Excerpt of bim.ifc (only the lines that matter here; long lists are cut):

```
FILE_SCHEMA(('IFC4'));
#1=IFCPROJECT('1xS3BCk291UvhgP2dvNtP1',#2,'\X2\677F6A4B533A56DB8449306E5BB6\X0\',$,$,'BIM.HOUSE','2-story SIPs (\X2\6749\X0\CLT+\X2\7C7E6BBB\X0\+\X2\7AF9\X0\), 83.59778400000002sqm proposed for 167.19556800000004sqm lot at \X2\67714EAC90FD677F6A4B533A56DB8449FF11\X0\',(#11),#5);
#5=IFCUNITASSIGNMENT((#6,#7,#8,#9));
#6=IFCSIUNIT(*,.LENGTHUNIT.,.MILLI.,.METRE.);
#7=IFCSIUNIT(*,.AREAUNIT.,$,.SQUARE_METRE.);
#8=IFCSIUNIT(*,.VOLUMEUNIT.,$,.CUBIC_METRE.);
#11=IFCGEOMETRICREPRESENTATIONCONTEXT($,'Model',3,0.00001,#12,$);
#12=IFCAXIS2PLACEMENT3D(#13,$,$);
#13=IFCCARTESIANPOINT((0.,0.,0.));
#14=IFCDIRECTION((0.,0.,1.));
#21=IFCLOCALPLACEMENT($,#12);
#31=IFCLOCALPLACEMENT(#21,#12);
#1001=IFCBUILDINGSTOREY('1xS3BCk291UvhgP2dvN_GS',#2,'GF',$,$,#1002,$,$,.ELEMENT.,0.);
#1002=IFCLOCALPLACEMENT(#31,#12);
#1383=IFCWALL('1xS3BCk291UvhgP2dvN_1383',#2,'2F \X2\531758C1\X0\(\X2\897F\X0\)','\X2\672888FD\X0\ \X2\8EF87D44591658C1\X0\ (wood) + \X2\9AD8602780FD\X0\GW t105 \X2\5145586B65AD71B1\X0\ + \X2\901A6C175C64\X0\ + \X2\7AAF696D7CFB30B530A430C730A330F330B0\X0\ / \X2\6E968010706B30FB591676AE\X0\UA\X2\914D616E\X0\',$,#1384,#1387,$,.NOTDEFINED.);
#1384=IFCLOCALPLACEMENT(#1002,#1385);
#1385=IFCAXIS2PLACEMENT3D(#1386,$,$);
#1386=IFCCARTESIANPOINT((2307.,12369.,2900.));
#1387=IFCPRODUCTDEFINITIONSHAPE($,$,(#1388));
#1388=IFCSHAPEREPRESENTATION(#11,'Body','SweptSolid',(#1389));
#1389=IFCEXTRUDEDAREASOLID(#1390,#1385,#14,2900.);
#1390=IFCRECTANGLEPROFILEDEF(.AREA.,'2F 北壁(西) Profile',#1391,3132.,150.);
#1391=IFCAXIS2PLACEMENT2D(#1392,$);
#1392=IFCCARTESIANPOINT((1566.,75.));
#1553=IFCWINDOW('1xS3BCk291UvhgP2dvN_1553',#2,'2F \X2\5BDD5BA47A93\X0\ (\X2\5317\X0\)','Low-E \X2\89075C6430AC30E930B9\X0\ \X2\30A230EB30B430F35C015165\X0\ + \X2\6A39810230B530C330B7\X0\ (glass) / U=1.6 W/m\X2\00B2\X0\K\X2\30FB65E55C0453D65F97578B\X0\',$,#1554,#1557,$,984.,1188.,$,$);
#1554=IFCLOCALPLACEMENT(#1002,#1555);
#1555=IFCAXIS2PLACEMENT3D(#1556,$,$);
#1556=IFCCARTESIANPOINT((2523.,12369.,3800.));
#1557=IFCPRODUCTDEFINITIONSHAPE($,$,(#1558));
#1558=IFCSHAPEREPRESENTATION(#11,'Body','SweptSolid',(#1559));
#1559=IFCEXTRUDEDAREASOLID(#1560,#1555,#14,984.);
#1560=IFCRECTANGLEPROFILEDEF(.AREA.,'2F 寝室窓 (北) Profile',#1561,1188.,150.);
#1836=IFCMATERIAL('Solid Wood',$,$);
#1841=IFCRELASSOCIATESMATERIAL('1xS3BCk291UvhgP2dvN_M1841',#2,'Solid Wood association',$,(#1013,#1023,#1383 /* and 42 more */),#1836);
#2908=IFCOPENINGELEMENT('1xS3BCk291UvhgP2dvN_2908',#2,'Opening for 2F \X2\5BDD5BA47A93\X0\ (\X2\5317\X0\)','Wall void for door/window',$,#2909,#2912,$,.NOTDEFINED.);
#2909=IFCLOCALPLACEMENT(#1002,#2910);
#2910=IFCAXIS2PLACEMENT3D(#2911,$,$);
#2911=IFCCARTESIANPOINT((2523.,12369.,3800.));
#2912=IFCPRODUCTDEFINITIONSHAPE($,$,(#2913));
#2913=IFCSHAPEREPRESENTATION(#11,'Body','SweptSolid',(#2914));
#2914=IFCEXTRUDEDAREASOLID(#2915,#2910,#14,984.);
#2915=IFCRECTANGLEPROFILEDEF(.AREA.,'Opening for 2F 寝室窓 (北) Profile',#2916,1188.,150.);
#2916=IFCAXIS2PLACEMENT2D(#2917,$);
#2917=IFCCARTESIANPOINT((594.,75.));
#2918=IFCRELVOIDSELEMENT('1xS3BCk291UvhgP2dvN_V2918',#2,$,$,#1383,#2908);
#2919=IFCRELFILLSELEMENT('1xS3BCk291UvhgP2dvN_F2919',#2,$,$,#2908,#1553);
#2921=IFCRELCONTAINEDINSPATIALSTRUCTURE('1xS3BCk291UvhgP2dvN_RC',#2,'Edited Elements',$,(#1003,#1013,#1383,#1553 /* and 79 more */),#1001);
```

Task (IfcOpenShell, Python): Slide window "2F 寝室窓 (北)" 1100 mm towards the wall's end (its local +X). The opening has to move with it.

```python
import ifcopenshell
import ifcopenshell.api.geometry
import ifcopenshell.util.placement
import ifcopenshell.util.unit

model = ifcopenshell.open("bim.ifc")
unit_scale = ifcopenshell.util.unit.calculate_unit_scale(model)

window = model.by_id(1553)
opening = window.FillsVoids[0].RelatingOpeningElement
wall = opening.VoidsElements[0].RelatingBuildingElement

wall_matrix = ifcopenshell.util.placement.get_local_placement(wall.ObjectPlacement)
shift = wall_matrix[:3, 0] * 1.1 / unit_scale
before = ifcopenshell.util.placement.get_local_placement(window.ObjectPlacement)[:3, 3].copy()

# The window is not placed relative to its opening, so move both.
for product in (opening, window):
    matrix = ifcopenshell.util.placement.get_local_placement(product.ObjectPlacement)
    matrix[:3, 3] += shift
    ifcopenshell.api.geometry.edit_object_placement(model, product=product, matrix=matrix, is_si=False)

after = ifcopenshell.util.placement.get_local_placement(window.ObjectPlacement)[:3, 3]
print("window moved by", (after - before).round(3) + 0.0)

model.write("bim_rev.ifc")
```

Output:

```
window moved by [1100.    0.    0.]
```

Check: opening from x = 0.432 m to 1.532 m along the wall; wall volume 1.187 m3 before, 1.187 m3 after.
